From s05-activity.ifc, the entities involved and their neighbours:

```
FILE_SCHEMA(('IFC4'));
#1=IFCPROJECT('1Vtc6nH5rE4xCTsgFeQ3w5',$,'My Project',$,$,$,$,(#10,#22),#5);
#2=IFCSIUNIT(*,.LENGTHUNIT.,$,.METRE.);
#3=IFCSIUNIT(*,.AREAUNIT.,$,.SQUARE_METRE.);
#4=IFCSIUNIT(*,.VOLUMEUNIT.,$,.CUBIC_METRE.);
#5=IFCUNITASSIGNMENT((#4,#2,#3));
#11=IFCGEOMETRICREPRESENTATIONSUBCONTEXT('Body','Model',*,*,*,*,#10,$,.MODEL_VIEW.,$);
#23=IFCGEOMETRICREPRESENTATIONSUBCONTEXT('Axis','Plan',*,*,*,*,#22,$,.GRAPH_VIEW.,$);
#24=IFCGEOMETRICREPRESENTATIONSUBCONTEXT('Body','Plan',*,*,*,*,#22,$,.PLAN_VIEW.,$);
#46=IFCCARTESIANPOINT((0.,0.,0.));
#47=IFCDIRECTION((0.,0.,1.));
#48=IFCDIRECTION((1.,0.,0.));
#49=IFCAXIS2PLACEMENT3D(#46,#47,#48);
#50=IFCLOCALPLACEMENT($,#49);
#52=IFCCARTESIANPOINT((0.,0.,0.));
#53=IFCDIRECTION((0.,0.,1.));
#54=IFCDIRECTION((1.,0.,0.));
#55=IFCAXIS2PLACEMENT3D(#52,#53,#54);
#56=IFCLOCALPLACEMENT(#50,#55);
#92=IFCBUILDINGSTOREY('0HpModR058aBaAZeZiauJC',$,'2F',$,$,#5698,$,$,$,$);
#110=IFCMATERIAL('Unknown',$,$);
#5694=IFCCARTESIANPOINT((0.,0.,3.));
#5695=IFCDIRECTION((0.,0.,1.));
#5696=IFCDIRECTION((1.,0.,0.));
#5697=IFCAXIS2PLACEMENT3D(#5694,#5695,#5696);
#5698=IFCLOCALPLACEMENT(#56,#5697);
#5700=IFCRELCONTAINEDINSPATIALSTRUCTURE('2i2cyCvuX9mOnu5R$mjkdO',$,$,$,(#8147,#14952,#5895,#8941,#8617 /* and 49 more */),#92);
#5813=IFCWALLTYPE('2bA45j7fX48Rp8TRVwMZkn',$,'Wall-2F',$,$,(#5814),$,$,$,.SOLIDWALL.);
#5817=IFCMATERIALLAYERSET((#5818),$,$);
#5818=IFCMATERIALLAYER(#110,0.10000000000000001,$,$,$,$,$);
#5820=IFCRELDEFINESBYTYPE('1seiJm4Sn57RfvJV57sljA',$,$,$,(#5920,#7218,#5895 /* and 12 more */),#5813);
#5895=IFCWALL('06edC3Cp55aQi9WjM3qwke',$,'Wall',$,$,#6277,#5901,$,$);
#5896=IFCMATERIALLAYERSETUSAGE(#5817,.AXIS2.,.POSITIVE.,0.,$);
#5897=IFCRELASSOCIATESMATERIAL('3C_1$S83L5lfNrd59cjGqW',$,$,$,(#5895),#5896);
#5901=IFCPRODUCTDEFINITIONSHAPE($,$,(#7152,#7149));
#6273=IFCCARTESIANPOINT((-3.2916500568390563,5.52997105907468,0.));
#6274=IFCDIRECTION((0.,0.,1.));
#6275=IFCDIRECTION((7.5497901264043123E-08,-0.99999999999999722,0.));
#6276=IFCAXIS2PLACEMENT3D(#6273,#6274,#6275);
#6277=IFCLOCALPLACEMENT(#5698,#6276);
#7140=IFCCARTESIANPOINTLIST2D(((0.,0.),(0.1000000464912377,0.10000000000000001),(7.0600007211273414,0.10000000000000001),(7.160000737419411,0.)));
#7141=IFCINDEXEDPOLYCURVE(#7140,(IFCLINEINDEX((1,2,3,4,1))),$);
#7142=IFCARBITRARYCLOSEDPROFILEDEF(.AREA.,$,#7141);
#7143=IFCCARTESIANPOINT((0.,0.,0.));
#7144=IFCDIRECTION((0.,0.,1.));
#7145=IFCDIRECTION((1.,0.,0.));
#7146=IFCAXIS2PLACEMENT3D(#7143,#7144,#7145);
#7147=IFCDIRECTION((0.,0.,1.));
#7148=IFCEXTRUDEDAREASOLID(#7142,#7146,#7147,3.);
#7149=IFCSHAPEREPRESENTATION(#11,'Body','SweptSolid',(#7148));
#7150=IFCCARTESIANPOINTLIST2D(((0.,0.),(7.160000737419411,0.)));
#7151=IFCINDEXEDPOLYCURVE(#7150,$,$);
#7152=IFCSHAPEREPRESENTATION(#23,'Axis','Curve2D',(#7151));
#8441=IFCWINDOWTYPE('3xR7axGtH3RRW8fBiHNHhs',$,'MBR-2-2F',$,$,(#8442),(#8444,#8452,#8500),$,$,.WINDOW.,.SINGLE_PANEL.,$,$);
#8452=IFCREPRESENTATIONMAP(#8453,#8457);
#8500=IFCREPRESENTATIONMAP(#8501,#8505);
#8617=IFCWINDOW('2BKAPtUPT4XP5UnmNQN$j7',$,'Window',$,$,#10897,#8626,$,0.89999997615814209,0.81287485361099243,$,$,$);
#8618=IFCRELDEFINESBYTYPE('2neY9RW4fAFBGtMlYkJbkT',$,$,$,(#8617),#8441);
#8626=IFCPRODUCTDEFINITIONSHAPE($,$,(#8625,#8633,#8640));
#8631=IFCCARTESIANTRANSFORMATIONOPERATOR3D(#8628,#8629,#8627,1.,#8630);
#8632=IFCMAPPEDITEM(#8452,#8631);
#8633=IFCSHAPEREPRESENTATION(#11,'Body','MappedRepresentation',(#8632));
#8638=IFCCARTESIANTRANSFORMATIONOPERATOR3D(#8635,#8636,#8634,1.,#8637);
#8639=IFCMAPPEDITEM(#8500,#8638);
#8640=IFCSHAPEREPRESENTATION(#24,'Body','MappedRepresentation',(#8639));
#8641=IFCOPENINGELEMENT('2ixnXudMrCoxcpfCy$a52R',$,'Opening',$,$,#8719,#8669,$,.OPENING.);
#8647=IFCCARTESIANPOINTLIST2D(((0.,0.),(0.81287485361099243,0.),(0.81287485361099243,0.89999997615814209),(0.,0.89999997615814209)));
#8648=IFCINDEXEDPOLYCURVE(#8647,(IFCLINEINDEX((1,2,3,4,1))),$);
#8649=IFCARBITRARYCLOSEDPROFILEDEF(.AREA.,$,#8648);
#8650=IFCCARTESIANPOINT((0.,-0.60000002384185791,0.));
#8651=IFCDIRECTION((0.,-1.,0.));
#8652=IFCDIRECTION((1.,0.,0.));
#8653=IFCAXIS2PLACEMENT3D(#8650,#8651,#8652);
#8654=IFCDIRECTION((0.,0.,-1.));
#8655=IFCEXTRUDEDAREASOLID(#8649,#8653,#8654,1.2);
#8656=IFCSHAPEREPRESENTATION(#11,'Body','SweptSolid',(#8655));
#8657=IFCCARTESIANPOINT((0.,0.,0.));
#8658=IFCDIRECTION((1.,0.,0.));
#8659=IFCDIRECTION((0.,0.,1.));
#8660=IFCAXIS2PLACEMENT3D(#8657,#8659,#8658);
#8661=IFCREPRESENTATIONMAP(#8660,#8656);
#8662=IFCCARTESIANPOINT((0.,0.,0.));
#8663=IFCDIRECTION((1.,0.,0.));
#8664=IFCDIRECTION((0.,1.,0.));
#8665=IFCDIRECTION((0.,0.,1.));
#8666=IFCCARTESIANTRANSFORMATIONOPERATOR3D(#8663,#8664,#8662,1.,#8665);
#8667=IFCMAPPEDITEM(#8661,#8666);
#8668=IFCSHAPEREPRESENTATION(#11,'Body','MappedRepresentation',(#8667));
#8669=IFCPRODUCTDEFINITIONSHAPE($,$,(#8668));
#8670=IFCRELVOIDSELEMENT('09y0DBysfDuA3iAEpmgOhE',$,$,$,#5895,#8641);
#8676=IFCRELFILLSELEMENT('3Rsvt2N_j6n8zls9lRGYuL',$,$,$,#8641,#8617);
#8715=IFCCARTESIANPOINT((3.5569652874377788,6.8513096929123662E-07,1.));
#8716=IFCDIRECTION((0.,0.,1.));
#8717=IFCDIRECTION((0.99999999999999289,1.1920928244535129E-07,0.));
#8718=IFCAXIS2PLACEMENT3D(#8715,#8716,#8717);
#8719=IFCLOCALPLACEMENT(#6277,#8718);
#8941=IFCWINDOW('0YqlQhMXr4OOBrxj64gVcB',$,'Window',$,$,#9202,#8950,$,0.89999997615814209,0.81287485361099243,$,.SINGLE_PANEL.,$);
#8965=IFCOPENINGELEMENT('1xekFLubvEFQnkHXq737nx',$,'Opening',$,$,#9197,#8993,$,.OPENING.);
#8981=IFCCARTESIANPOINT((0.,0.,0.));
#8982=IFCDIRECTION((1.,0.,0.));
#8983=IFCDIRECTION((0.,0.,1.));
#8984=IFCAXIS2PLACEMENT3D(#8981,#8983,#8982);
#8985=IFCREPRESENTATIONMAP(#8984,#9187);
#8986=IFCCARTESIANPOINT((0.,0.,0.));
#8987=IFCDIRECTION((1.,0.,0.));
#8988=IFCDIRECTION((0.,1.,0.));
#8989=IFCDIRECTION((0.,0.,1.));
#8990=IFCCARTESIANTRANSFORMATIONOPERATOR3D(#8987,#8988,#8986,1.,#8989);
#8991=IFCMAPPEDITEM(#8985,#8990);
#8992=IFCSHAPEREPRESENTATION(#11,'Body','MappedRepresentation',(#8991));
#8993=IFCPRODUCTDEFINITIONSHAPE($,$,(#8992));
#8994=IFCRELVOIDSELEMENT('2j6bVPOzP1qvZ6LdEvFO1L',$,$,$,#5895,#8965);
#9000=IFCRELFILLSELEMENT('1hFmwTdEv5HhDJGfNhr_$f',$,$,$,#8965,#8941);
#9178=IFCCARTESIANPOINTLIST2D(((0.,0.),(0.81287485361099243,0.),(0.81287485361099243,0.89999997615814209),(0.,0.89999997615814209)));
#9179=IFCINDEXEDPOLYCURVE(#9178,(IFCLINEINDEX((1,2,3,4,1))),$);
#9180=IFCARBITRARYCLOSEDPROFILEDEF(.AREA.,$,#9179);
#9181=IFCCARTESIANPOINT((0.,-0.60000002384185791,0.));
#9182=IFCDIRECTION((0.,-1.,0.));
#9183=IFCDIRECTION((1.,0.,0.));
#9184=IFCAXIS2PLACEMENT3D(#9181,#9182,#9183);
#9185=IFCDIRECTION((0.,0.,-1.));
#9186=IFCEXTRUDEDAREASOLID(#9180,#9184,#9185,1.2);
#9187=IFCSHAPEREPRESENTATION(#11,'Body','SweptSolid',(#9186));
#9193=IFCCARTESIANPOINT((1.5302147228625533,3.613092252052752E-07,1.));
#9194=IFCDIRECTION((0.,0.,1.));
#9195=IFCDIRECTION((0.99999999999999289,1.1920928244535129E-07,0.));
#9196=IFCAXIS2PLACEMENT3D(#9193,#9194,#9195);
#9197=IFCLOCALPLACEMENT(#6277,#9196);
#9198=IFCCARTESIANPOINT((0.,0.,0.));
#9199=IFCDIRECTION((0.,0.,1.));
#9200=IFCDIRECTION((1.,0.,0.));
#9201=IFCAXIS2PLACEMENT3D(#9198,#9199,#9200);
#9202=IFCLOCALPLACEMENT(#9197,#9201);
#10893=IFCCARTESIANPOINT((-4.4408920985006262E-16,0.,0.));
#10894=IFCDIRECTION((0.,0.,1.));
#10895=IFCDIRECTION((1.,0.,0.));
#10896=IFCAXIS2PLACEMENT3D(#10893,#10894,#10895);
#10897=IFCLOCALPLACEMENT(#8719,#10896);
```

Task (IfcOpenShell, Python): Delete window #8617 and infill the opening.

```python
import ifcopenshell
import ifcopenshell.api.feature
import ifcopenshell.api.root
import ifcopenshell.geom
import ifcopenshell.util.shape

model = ifcopenshell.open("s05-activity.ifc")
settings = ifcopenshell.geom.settings()


def volume(element):
    """Net volume in cubic metres, openings subtracted."""
    shape = ifcopenshell.geom.create_shape(settings, element)
    return ifcopenshell.util.shape.get_volume(shape.geometry)


window = model.by_guid("2BKAPtUPT4XP5UnmNQN$j7")
opening = window.FillsVoids[0].RelatingOpeningElement
wall = opening.VoidsElements[0].RelatingBuildingElement
before = volume(wall)

ifcopenshell.api.root.remove_product(model, product=window)
ifcopenshell.api.feature.remove_feature(model, feature=opening)

after = volume(wall)

print(f"wall volume {before:.3f} -> {after:.3f} m3")

model.write("s05-activity-out.ifc")
```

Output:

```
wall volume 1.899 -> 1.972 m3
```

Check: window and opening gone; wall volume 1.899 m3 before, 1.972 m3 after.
